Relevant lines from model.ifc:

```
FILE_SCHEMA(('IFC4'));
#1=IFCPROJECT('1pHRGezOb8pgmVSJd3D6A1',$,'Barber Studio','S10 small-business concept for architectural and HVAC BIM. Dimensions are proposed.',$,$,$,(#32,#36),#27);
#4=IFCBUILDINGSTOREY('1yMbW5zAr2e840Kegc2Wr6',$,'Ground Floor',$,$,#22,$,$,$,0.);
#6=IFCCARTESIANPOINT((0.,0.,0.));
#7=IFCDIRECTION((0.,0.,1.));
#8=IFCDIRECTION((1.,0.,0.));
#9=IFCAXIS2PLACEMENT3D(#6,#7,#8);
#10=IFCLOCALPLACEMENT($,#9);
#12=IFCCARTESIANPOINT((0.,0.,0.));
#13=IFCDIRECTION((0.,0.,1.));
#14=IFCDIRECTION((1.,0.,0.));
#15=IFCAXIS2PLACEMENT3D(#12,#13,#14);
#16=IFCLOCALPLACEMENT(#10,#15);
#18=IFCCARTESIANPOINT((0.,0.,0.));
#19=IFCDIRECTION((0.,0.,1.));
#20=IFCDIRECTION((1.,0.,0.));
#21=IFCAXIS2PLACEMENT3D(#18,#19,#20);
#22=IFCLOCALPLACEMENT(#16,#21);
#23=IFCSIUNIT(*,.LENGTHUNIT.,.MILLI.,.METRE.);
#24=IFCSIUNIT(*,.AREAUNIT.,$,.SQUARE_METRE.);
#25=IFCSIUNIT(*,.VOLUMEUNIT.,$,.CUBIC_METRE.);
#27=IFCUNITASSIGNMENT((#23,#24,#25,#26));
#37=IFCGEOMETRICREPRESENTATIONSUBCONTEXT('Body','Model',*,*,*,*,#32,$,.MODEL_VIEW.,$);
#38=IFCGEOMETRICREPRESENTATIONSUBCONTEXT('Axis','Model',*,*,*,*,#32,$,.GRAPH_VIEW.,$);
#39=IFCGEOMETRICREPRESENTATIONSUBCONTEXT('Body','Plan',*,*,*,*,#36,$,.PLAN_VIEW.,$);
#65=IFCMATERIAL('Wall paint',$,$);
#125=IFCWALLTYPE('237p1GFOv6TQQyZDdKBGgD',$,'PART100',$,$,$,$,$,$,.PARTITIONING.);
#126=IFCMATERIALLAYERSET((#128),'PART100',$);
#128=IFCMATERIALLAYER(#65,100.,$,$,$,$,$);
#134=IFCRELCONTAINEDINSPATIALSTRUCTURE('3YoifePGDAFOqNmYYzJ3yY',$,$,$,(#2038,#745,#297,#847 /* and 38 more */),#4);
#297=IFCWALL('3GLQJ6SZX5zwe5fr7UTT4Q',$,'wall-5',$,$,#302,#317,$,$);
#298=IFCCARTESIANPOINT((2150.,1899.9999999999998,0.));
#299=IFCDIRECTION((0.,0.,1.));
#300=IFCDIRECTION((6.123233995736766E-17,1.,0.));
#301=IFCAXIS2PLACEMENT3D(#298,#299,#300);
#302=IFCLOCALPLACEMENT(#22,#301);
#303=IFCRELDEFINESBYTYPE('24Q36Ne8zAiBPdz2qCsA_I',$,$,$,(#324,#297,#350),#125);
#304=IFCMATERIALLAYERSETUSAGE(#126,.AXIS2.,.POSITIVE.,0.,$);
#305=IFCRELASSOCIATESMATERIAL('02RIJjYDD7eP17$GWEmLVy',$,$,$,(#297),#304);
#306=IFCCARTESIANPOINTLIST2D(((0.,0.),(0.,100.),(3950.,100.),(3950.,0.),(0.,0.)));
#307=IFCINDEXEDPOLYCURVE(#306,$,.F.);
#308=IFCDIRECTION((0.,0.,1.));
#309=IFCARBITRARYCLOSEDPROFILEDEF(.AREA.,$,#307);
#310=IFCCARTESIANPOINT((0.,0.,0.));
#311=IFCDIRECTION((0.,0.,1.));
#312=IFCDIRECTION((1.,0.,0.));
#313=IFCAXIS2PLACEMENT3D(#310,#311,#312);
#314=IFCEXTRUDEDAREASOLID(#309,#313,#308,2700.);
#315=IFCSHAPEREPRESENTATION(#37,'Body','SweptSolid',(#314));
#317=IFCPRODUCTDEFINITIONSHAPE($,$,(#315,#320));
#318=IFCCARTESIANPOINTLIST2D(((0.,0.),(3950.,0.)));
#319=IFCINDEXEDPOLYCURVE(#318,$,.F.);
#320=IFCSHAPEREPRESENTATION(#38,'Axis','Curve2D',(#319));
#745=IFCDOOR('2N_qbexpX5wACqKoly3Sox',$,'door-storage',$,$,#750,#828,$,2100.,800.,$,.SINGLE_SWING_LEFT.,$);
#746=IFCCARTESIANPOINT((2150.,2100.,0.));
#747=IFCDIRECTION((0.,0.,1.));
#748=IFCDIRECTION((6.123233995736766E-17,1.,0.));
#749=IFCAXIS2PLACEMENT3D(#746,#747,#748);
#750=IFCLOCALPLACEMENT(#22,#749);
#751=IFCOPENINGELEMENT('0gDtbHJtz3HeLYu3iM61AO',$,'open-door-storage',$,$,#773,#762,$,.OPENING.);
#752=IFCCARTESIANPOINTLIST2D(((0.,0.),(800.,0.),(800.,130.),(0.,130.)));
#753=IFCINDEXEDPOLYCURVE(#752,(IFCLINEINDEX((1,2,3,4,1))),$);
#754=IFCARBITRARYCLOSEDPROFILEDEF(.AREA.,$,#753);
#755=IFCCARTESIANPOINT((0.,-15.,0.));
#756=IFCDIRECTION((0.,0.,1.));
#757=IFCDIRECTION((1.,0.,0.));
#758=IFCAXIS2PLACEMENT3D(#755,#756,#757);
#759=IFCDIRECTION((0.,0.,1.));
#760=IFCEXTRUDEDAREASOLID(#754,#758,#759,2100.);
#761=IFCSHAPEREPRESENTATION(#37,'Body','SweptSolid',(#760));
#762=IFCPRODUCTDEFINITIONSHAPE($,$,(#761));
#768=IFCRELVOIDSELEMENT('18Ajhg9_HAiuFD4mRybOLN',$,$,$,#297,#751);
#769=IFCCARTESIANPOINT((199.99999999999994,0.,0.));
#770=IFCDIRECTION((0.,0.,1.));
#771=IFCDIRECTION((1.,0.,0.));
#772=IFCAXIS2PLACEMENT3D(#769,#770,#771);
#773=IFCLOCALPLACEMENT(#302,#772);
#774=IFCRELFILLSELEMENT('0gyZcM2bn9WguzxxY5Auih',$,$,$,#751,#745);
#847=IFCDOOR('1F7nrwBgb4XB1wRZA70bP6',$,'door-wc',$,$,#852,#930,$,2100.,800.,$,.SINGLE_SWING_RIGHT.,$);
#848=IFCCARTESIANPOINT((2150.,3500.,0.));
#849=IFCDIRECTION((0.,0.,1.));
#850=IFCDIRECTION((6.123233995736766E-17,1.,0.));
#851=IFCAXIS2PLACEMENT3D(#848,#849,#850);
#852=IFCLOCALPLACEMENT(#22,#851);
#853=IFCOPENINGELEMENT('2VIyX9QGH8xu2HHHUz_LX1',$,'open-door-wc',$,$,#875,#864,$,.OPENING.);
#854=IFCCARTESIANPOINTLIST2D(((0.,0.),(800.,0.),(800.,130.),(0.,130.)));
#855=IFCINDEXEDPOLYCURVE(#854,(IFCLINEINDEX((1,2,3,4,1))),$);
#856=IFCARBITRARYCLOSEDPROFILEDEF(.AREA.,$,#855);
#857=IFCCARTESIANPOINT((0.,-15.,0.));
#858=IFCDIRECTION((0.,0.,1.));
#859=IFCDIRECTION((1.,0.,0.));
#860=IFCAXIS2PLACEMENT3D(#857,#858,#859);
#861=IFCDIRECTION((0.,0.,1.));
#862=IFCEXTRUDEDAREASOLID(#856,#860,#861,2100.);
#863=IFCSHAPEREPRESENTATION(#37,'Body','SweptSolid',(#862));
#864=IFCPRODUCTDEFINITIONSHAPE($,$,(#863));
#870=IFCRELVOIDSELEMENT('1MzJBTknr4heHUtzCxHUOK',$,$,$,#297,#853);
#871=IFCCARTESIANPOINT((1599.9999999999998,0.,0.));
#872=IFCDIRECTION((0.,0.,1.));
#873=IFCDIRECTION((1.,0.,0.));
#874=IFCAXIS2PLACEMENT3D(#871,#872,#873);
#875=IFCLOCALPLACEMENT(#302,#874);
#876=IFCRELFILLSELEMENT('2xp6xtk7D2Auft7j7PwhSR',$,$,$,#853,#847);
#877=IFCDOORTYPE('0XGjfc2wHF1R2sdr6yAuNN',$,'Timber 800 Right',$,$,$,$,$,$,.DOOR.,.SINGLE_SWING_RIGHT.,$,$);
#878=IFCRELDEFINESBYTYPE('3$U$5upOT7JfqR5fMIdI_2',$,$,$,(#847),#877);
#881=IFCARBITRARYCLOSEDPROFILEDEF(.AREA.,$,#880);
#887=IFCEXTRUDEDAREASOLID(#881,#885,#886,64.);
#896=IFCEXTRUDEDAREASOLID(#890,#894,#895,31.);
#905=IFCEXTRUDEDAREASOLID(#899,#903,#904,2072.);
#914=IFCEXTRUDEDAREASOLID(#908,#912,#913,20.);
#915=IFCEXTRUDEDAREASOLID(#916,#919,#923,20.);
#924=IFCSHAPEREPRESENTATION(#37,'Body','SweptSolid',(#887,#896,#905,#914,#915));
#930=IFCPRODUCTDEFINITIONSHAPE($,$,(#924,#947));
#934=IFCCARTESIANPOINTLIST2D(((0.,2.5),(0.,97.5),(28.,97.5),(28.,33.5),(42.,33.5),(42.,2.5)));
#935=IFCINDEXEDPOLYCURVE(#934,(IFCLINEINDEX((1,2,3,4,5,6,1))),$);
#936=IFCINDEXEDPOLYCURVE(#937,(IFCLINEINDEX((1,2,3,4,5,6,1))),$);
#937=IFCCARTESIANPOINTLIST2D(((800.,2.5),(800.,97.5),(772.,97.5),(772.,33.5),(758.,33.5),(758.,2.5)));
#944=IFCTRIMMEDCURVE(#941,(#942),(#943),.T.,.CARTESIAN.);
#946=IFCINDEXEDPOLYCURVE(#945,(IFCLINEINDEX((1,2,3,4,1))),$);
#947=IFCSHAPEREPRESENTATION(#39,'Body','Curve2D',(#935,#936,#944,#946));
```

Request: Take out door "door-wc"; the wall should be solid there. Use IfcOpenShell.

```python
import ifcopenshell
import ifcopenshell.api.feature
import ifcopenshell.api.root
import ifcopenshell.geom
import ifcopenshell.util.shape

model = ifcopenshell.open("model.ifc")
settings = ifcopenshell.geom.settings()


def volume(element):
    """Net volume in cubic metres, openings subtracted."""
    shape = ifcopenshell.geom.create_shape(settings, element)
    return ifcopenshell.util.shape.get_volume(shape.geometry)


door = model.by_guid("1F7nrwBgb4XB1wRZA70bP6")
opening = door.FillsVoids[0].RelatingOpeningElement
wall = opening.VoidsElements[0].RelatingBuildingElement
before = volume(wall)

ifcopenshell.api.root.remove_product(model, product=door)
ifcopenshell.api.feature.remove_feature(model, feature=opening)

after = volume(wall)

print(f"wall volume {before:.3f} -> {after:.3f} m3")

model.write("model_v2.ifc")
```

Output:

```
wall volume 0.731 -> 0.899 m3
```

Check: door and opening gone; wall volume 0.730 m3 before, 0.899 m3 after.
